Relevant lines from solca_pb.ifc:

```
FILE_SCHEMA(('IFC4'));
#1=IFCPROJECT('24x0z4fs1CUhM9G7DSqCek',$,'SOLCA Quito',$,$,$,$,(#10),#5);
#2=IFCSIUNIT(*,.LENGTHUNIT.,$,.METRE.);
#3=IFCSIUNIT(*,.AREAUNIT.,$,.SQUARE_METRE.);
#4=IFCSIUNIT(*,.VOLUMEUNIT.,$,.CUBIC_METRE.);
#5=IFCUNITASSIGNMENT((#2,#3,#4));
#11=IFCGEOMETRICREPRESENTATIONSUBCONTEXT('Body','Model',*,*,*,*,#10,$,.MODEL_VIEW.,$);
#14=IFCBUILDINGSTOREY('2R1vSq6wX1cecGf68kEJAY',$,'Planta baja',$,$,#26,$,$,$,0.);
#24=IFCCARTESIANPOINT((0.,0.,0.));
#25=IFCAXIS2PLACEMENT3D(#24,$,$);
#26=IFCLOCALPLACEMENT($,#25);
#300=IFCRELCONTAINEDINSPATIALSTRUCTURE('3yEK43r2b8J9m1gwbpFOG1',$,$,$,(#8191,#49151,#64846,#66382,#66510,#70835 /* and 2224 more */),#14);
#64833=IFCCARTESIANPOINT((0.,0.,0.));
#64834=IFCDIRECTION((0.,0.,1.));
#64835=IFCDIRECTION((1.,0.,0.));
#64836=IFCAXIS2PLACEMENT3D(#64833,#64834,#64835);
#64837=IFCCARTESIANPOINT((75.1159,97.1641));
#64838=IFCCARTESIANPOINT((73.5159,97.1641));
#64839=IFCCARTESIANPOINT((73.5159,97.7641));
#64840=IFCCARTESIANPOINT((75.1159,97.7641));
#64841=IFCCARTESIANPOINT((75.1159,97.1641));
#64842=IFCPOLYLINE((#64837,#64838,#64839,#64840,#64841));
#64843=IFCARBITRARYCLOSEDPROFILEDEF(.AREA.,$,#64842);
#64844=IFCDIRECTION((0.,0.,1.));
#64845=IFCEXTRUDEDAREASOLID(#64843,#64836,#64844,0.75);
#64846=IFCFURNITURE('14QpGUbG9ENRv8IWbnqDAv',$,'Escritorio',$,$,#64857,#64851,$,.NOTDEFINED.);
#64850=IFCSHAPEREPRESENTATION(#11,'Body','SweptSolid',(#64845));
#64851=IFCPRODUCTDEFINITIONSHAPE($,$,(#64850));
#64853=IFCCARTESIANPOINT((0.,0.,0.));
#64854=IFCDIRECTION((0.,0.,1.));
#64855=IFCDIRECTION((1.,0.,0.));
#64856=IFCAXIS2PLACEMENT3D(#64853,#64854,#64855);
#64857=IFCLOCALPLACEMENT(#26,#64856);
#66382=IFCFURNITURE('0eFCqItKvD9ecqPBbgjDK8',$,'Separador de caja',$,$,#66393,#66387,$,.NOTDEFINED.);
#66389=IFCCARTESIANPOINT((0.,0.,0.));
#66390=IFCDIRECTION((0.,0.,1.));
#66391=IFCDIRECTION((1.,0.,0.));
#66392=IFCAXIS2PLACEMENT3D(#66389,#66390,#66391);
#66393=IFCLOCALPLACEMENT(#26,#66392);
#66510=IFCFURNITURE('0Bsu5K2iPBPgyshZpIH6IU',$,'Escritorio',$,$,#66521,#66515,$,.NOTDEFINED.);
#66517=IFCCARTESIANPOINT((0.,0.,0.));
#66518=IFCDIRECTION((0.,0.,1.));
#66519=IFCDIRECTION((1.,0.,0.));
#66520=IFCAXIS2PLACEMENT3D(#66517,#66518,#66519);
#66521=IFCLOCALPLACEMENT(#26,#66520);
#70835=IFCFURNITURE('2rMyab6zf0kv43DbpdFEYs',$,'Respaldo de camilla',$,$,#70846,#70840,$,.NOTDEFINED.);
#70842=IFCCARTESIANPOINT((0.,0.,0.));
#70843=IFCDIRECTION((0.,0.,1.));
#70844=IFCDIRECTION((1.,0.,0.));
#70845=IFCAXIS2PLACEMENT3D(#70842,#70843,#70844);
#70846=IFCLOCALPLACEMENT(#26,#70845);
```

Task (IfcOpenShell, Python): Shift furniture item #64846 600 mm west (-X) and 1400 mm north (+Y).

```python
import ifcopenshell
import ifcopenshell.api.geometry
import ifcopenshell.util.placement
import ifcopenshell.util.unit

model = ifcopenshell.open("solca_pb.ifc")
unit_scale = ifcopenshell.util.unit.calculate_unit_scale(model)

item = model.by_guid("14QpGUbG9ENRv8IWbnqDAv")
matrix = ifcopenshell.util.placement.get_local_placement(item.ObjectPlacement)
matrix[0, 3] -= 0.6 / unit_scale
matrix[1, 3] += 1.4 / unit_scale
ifcopenshell.api.geometry.edit_object_placement(model, product=item, matrix=matrix, is_si=False)

print(ifcopenshell.util.placement.get_local_placement(item.ObjectPlacement).round(3) + 0.0)

model.write("solca_pb_rev.ifc")
```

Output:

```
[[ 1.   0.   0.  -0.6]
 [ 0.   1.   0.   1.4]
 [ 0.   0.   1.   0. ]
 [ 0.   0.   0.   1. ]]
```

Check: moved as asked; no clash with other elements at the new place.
